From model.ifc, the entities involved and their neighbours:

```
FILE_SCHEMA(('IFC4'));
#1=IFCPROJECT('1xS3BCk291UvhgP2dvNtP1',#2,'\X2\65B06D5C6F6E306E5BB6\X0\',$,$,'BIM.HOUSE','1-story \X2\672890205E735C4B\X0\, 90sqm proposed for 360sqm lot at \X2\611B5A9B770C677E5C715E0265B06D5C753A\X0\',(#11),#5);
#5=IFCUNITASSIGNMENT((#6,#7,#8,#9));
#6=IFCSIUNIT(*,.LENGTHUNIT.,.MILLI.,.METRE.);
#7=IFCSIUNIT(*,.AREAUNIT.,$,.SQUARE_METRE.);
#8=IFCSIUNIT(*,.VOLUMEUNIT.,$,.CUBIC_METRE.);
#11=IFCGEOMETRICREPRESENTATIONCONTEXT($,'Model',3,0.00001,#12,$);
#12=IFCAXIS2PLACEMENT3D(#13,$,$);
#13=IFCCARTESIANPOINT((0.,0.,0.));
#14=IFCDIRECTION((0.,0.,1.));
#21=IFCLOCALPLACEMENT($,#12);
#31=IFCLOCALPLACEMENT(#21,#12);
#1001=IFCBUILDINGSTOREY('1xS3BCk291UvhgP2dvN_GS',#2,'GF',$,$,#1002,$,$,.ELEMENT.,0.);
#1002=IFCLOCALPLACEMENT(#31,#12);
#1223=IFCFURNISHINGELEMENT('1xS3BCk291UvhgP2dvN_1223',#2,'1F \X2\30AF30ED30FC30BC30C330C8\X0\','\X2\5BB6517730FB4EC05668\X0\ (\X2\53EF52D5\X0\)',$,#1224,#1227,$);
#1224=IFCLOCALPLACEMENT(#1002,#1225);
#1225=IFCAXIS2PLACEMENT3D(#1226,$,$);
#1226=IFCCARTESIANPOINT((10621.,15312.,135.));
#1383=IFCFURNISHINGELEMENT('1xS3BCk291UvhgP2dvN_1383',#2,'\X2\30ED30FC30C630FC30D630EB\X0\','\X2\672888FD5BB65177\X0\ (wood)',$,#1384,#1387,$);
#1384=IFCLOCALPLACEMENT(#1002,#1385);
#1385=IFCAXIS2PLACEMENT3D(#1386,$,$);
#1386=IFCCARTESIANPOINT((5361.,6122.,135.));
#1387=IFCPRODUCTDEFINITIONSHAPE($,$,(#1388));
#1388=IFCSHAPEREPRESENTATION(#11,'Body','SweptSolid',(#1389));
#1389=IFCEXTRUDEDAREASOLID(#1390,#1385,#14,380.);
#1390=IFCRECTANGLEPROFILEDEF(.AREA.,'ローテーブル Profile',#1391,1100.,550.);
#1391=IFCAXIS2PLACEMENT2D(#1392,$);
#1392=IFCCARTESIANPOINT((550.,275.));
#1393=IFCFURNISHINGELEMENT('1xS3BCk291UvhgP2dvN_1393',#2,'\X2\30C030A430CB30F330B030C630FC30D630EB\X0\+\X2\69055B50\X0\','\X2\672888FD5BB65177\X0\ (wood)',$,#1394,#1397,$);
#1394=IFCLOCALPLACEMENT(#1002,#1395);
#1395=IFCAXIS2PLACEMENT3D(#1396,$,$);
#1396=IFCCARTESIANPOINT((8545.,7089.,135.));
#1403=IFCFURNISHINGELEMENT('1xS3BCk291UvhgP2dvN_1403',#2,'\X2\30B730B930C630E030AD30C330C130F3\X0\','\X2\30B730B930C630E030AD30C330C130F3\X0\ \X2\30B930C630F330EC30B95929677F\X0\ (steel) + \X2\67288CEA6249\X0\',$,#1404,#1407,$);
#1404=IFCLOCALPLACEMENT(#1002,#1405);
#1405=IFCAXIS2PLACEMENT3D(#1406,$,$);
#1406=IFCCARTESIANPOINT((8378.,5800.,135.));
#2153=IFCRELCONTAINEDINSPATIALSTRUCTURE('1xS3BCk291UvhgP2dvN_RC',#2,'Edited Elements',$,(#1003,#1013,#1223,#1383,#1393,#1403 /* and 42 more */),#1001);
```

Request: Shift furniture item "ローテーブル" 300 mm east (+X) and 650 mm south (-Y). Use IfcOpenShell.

```python
import ifcopenshell
import ifcopenshell.api.geometry
import ifcopenshell.util.placement

model = ifcopenshell.open("model.ifc")

item = model.by_guid("1xS3BCk291UvhgP2dvN_1383")
matrix = ifcopenshell.util.placement.get_local_placement(item.ObjectPlacement)
matrix[0, 3] += 300.0
matrix[1, 3] -= 650.0
ifcopenshell.api.geometry.edit_object_placement(model, product=item, matrix=matrix, is_si=False)

print(ifcopenshell.util.placement.get_local_placement(item.ObjectPlacement).round(3) + 0.0)

model.write("model_v2.ifc")
```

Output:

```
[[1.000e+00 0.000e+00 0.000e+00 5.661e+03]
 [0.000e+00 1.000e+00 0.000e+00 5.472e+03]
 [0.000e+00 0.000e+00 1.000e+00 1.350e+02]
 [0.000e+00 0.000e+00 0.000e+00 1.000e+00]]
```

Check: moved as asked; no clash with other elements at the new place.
